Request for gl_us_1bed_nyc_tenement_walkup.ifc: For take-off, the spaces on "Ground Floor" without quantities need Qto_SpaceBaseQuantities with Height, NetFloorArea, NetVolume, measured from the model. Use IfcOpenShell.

First a look at what the model holds.

```python
import ifcopenshell
import ifcopenshell.util.element
import ifcopenshell.util.unit

model = ifcopenshell.open("gl_us_1bed_nyc_tenement_walkup.ifc")
print(model.schema)
for unit_type in ("LENGTHUNIT", "AREAUNIT", "VOLUMEUNIT"):
    print(unit_type, ifcopenshell.util.unit.calculate_unit_scale(model, unit_type))
storey = next(s for s in model.by_type("IfcBuildingStorey") if s.Name == "Ground Floor")
spaces = [e for e in ifcopenshell.util.element.get_decomposition(storey) if e.is_a("IfcSpace")]
for e in sorted(spaces, key=lambda e: e.id()):
    print(e.id(), e.is_a(), e.Name, list(ifcopenshell.util.element.get_psets(e, qtos_only=True)), sep=" | ")
```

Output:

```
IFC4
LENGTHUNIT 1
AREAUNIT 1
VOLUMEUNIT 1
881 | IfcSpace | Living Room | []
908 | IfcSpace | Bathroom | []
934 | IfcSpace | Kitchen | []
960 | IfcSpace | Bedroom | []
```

```python
import ifcopenshell
import ifcopenshell.api.pset
import ifcopenshell.geom
import ifcopenshell.util.element
import ifcopenshell.util.shape
import ifcopenshell.util.unit

model = ifcopenshell.open("gl_us_1bed_nyc_tenement_walkup.ifc")
unit_scale = ifcopenshell.util.unit.calculate_unit_scale(model)
area_scale = ifcopenshell.util.unit.calculate_unit_scale(model, "AREAUNIT")
volume_scale = ifcopenshell.util.unit.calculate_unit_scale(model, "VOLUMEUNIT")
settings = ifcopenshell.geom.settings()

storey = next(s for s in model.by_type("IfcBuildingStorey") if s.Name == "Ground Floor")
spaces = [e for e in ifcopenshell.util.element.get_decomposition(storey) if e.is_a("IfcSpace")]

for e in sorted(spaces, key=lambda e: e.id()):
    if ifcopenshell.util.element.get_psets(e, qtos_only=True, should_inherit=False):
        continue
    # Geometry comes back in metres, in the element's own axes.
    shape = ifcopenshell.geom.create_shape(settings, e)
    values = {
        "Height": ifcopenshell.util.shape.get_z(shape.geometry) / unit_scale,
        "NetFloorArea": ifcopenshell.util.shape.get_footprint_area(shape.geometry) / area_scale,
        "NetVolume": ifcopenshell.util.shape.get_volume(shape.geometry) / volume_scale,
    }
    qto = ifcopenshell.api.pset.add_qto(model, product=e, name="Qto_SpaceBaseQuantities")
    ifcopenshell.api.pset.edit_qto(model, qto=qto, properties=values)
    print(e.id(), {k: round(v, 3) for k, v in values.items()})

model.write("gl_us_1bed_nyc_tenement_walkup_edited.ifc")
```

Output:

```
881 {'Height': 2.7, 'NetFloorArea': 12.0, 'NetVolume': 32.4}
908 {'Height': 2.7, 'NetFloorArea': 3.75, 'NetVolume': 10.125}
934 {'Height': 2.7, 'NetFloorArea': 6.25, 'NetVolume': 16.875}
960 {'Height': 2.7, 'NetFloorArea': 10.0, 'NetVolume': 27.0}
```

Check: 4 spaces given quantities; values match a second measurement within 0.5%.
